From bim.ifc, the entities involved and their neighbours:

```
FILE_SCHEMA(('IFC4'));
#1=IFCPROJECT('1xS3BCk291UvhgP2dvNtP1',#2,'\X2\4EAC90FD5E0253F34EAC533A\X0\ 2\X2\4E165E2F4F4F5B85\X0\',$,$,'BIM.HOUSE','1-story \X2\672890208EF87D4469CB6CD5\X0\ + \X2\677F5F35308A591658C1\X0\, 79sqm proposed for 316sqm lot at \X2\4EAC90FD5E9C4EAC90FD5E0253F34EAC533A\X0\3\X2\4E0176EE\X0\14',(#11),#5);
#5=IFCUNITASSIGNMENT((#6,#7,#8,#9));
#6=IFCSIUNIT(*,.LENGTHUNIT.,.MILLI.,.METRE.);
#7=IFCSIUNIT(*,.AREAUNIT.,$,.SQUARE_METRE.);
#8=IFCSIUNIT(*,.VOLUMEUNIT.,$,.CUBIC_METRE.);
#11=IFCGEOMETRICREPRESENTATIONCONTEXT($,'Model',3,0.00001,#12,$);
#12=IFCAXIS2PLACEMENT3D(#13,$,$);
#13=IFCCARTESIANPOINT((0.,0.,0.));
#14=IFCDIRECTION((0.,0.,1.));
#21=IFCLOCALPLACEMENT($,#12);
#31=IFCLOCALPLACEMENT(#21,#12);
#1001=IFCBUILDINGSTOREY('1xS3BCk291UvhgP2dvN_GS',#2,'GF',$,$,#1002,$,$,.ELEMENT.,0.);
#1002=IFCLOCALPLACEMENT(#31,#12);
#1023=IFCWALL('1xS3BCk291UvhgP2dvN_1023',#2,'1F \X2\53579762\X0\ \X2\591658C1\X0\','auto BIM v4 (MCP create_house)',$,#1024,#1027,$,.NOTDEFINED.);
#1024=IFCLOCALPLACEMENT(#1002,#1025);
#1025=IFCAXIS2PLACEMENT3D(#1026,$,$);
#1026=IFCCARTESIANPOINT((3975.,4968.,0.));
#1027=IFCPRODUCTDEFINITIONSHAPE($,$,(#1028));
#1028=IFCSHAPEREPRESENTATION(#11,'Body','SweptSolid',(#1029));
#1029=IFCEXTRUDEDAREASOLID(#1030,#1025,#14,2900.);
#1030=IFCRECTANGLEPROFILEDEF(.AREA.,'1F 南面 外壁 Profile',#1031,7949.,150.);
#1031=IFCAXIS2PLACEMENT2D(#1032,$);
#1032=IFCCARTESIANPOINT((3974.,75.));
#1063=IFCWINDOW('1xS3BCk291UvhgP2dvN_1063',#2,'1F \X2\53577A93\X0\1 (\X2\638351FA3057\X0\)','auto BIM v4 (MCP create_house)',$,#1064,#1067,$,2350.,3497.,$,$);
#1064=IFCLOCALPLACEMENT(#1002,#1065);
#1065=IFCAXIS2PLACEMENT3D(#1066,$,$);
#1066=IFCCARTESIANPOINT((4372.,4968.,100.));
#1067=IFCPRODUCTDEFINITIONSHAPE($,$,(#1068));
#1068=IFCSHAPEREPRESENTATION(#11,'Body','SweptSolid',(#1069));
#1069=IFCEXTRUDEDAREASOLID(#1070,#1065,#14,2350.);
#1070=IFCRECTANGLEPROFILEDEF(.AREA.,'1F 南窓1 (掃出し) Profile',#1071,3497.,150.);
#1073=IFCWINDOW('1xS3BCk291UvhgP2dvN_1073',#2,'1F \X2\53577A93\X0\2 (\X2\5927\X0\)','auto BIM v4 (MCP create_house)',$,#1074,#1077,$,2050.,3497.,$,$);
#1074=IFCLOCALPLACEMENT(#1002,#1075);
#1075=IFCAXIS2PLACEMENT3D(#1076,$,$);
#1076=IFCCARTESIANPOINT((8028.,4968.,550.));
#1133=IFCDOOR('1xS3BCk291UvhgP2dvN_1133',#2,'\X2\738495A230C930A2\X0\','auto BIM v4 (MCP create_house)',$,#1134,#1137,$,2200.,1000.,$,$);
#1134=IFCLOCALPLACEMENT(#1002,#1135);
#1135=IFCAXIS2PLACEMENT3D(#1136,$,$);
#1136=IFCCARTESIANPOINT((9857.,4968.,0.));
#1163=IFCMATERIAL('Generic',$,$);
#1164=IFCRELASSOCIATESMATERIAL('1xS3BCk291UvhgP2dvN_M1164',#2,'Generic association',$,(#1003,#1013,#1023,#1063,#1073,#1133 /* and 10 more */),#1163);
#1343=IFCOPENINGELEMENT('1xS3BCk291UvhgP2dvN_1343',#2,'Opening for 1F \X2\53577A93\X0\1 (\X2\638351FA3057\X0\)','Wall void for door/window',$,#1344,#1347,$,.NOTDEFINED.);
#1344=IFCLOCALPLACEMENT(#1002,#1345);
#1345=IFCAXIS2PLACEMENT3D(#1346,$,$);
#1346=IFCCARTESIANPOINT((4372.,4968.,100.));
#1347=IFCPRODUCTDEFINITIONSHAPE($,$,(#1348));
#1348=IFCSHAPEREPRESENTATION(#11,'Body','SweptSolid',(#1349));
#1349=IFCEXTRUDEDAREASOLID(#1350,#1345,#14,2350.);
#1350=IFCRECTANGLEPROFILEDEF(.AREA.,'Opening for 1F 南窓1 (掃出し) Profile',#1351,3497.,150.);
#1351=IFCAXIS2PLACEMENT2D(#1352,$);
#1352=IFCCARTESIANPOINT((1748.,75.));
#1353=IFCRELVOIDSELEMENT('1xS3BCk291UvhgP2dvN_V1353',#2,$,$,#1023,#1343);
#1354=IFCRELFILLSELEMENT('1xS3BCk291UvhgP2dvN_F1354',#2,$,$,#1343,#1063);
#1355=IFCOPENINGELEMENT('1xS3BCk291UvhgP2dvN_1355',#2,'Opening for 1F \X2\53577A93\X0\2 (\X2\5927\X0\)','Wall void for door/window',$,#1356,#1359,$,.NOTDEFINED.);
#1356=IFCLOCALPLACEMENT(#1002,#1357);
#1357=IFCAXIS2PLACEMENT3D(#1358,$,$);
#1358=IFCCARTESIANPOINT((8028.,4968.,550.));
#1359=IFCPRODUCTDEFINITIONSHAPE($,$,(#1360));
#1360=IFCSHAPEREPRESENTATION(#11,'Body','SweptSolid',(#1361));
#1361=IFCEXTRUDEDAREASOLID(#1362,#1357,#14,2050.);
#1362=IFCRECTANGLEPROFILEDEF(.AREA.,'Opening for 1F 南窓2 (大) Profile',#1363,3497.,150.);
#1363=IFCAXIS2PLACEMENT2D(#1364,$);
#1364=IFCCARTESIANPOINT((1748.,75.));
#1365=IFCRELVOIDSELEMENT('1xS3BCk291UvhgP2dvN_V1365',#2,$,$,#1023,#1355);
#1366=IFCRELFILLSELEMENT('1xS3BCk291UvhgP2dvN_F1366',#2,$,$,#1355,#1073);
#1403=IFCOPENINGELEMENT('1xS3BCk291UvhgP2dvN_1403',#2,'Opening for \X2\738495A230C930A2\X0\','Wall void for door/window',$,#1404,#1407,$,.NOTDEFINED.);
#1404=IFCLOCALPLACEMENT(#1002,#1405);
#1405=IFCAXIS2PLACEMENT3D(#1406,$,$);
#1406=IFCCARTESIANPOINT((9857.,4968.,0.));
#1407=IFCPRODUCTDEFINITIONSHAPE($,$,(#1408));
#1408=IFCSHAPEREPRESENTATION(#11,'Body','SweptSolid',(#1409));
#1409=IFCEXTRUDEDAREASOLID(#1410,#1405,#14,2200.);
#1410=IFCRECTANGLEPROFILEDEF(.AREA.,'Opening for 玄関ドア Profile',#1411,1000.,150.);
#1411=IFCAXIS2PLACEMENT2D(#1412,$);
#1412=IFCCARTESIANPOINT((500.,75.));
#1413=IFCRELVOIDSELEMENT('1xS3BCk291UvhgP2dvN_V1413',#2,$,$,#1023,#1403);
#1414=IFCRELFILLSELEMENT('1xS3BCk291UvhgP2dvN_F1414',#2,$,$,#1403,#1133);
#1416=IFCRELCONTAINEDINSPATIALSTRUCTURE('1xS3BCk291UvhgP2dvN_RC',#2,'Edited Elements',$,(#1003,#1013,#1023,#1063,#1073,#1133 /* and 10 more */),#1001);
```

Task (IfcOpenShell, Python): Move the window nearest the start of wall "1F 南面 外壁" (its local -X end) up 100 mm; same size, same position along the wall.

```python
import numpy as np
import ifcopenshell
import ifcopenshell.api.geometry
import ifcopenshell.util.placement
import ifcopenshell.util.unit

model = ifcopenshell.open("bim.ifc")
unit_scale = ifcopenshell.util.unit.calculate_unit_scale(model)

window = model.by_guid("1xS3BCk291UvhgP2dvN_1063")
opening = window.FillsVoids[0].RelatingOpeningElement
dz = 0.1 / unit_scale

shift = np.array([0.0, 0.0, dz])
# The window is not placed relative to its opening, so move both.
for product in (opening, window):
    matrix = ifcopenshell.util.placement.get_local_placement(product.ObjectPlacement)
    matrix[:3, 3] += shift
    ifcopenshell.api.geometry.edit_object_placement(model, product=product, matrix=matrix, is_si=False)

print(f"moved by {dz * unit_scale:+.3f} m")

model.write("bim_rev.ifc")
```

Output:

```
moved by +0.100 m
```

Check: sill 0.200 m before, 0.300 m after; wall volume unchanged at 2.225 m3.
